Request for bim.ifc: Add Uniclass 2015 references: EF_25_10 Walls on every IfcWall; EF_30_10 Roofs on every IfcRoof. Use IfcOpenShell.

First a look at what the model holds.

```python
import ifcopenshell

model = ifcopenshell.open("bim.ifc")
print(model.schema)
print("classifications:", [c.Name for c in model.by_type("IfcClassification")])
for ifc_class in ("IfcDoor", "IfcRoof", "IfcStair", "IfcWall", "IfcWindow"):
    print(ifc_class, len(model.by_type(ifc_class)))
```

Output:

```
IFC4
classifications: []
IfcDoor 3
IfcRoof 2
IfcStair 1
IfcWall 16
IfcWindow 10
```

```python
import ifcopenshell
import ifcopenshell.api.classification

model = ifcopenshell.open("bim.ifc")

system = ifcopenshell.api.classification.add_classification(model, classification="Uniclass 2015")

codes = {
    "IfcWall": ("EF_25_10", "Walls"),
    "IfcRoof": ("EF_30_10", "Roofs"),
}
for ifc_class, (code, name) in codes.items():
    products = model.by_type(ifc_class)
    ifcopenshell.api.classification.add_reference(
        model, products=products, classification=system, identification=code, name=name
    )
    print(code, len(products))

model.write("bim_edited.ifc")
```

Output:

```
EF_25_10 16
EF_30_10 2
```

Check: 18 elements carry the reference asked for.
